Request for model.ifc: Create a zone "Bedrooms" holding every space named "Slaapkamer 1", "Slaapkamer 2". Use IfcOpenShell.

First a look at what the model holds.

```python
import ifcopenshell

model = ifcopenshell.open("model.ifc")
print(model.schema)
seen = {}
for space in model.by_type("IfcSpace"):
    seen[space.LongName] = seen.get(space.LongName, 0) + 1
for name, count in sorted(seen.items(), key=str):
    print(count, "x", name)
print("zones:", [z.Name for z in model.by_type("IfcZone")][:20])
```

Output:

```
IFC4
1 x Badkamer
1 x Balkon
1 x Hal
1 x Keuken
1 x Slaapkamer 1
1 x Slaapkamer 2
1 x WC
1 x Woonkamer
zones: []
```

```python
import ifcopenshell
import ifcopenshell.api.group
import ifcopenshell.api.root

model = ifcopenshell.open("model.ifc")

names = {"Slaapkamer 1", "Slaapkamer 2"}
spaces = [s for s in model.by_type("IfcSpace") if s.LongName in names]

zone = ifcopenshell.api.root.create_entity(model, ifc_class="IfcZone", name="Bedrooms")
ifcopenshell.api.group.assign_group(model, products=spaces, group=zone)
print(len(spaces), "spaces in", zone.Name)

model.write("model_edited.ifc")
```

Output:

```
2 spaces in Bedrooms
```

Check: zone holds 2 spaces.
